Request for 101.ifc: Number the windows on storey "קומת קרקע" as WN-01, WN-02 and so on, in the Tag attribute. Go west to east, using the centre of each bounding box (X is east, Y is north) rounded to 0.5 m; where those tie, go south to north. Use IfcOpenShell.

First a look at what the model holds.

```python
import ifcopenshell
import ifcopenshell.util.element
import ifcopenshell.util.placement

model = ifcopenshell.open("101.ifc")
print(model.schema)
storey = next(s for s in model.by_type("IfcBuildingStorey") if s.Name == "קומת קרקע")
windows = [e for e in ifcopenshell.util.element.get_decomposition(storey) if e.is_a("IfcWindow")]
for e in sorted(windows, key=lambda e: e.id()):
    origin = ifcopenshell.util.placement.get_local_placement(e.ObjectPlacement)[:3, 3]
    print(e.id(), e.Tag, e.Name, origin.round(2) + 0.0, sep=" | ")
```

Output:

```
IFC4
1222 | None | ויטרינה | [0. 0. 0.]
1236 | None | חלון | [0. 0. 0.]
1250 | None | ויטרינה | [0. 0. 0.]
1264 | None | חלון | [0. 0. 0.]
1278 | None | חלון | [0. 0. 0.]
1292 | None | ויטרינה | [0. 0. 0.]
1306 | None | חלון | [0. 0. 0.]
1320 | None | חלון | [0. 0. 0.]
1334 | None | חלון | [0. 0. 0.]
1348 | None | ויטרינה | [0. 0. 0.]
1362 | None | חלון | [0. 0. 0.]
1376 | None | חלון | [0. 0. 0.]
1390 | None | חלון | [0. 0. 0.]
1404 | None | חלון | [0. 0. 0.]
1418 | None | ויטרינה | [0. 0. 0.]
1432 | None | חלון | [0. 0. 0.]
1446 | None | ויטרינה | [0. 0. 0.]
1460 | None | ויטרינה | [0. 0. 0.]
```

```python
import ifcopenshell
import ifcopenshell.geom
import ifcopenshell.util.element
import ifcopenshell.util.shape

model = ifcopenshell.open("101.ifc")
settings = ifcopenshell.geom.settings()
settings.set("use-world-coords", True)


def centre(element):
    shape = ifcopenshell.geom.create_shape(settings, element)
    return ifcopenshell.util.shape.get_bbox_centroid(shape.geometry)


storey = next(s for s in model.by_type("IfcBuildingStorey") if s.Name == "קומת קרקע")
windows = [e for e in ifcopenshell.util.element.get_decomposition(storey) if e.is_a("IfcWindow")]

# Insertion points can sit at a corner or the storey origin, so sort by the geometry (in metres).
centres = {e: centre(e) for e in windows}
windows.sort(key=lambda e: (round(centres[e][0] / 0.5), centres[e][1]))

for i, e in enumerate(windows, start=1):
    number = f"WN-{i:02d}"
    e.Tag = number
    print(e.id(), number)

model.write("101_edited.ifc")
```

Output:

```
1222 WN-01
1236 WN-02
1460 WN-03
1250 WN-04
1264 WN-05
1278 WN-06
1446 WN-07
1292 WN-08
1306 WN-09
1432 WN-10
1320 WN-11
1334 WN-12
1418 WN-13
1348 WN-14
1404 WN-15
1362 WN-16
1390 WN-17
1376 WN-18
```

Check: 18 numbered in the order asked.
